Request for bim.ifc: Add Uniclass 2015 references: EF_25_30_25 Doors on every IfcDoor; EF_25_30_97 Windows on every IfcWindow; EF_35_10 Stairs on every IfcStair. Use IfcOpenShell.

First a look at what the model holds.

```python
import ifcopenshell

model = ifcopenshell.open("bim.ifc")
print(model.schema)
print("classifications:", [c.Name for c in model.by_type("IfcClassification")])
for ifc_class in ("IfcDoor", "IfcRoof", "IfcStair", "IfcWall", "IfcWindow"):
    print(ifc_class, len(model.by_type(ifc_class)))
```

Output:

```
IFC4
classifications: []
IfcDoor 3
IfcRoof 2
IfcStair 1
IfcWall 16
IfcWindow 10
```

```python
import ifcopenshell
import ifcopenshell.api.classification

model = ifcopenshell.open("bim.ifc")

system = ifcopenshell.api.classification.add_classification(model, classification="Uniclass 2015")

codes = {
    "IfcDoor": ("EF_25_30_25", "Doors"),
    "IfcWindow": ("EF_25_30_97", "Windows"),
    "IfcStair": ("EF_35_10", "Stairs"),
}
for ifc_class, (code, name) in codes.items():
    products = model.by_type(ifc_class)
    ifcopenshell.api.classification.add_reference(
        model, products=products, classification=system, identification=code, name=name
    )
    print(code, len(products))

model.write("bim_edited.ifc")
```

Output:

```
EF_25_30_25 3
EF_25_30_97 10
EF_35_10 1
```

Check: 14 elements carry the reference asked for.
